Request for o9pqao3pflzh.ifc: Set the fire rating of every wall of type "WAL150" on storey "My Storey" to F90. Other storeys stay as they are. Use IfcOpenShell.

First a look at what the model holds.

```python
import ifcopenshell
import ifcopenshell.util.element

model = ifcopenshell.open("o9pqao3pflzh.ifc")
print(model.schema)
storey = next(s for s in model.by_type("IfcBuildingStorey") if s.Name == "My Storey")
walls = [e for e in ifcopenshell.util.element.get_decomposition(storey) if e.is_a("IfcWall")]
seen = {}
for e in walls:
    element_type = ifcopenshell.util.element.get_type(e)
    key = (element_type.Name if element_type != e and element_type else None, ifcopenshell.util.element.get_pset(e, "Pset_WallCommon", "FireRating"))
    seen[key] = seen.get(key, 0) + 1
for (name, value), count in sorted(seen.items(), key=str):
    print(count, "x", name, "|", value)
```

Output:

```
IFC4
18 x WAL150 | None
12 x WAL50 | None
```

```python
import ifcopenshell
import ifcopenshell.api.pset
import ifcopenshell.util.element

model = ifcopenshell.open("o9pqao3pflzh.ifc")

storey = next(s for s in model.by_type("IfcBuildingStorey") if s.Name == "My Storey")
walls = [e for e in ifcopenshell.util.element.get_decomposition(storey) if e.is_a("IfcWall")]

count = 0
for e in walls:
    element_type = ifcopenshell.util.element.get_type(e)
    if element_type in (None, e) or element_type.Name != "WAL150":
        continue
    # add_pset returns the element's existing set when there is one.
    pset = ifcopenshell.api.pset.add_pset(model, product=e, name="Pset_WallCommon")
    ifcopenshell.api.pset.edit_pset(model, pset=pset, properties={"FireRating": "F90"})
    count += 1

print(count, "walls updated")

model.write("o9pqao3pflzh_v2.ifc")
```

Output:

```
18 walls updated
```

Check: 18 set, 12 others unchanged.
